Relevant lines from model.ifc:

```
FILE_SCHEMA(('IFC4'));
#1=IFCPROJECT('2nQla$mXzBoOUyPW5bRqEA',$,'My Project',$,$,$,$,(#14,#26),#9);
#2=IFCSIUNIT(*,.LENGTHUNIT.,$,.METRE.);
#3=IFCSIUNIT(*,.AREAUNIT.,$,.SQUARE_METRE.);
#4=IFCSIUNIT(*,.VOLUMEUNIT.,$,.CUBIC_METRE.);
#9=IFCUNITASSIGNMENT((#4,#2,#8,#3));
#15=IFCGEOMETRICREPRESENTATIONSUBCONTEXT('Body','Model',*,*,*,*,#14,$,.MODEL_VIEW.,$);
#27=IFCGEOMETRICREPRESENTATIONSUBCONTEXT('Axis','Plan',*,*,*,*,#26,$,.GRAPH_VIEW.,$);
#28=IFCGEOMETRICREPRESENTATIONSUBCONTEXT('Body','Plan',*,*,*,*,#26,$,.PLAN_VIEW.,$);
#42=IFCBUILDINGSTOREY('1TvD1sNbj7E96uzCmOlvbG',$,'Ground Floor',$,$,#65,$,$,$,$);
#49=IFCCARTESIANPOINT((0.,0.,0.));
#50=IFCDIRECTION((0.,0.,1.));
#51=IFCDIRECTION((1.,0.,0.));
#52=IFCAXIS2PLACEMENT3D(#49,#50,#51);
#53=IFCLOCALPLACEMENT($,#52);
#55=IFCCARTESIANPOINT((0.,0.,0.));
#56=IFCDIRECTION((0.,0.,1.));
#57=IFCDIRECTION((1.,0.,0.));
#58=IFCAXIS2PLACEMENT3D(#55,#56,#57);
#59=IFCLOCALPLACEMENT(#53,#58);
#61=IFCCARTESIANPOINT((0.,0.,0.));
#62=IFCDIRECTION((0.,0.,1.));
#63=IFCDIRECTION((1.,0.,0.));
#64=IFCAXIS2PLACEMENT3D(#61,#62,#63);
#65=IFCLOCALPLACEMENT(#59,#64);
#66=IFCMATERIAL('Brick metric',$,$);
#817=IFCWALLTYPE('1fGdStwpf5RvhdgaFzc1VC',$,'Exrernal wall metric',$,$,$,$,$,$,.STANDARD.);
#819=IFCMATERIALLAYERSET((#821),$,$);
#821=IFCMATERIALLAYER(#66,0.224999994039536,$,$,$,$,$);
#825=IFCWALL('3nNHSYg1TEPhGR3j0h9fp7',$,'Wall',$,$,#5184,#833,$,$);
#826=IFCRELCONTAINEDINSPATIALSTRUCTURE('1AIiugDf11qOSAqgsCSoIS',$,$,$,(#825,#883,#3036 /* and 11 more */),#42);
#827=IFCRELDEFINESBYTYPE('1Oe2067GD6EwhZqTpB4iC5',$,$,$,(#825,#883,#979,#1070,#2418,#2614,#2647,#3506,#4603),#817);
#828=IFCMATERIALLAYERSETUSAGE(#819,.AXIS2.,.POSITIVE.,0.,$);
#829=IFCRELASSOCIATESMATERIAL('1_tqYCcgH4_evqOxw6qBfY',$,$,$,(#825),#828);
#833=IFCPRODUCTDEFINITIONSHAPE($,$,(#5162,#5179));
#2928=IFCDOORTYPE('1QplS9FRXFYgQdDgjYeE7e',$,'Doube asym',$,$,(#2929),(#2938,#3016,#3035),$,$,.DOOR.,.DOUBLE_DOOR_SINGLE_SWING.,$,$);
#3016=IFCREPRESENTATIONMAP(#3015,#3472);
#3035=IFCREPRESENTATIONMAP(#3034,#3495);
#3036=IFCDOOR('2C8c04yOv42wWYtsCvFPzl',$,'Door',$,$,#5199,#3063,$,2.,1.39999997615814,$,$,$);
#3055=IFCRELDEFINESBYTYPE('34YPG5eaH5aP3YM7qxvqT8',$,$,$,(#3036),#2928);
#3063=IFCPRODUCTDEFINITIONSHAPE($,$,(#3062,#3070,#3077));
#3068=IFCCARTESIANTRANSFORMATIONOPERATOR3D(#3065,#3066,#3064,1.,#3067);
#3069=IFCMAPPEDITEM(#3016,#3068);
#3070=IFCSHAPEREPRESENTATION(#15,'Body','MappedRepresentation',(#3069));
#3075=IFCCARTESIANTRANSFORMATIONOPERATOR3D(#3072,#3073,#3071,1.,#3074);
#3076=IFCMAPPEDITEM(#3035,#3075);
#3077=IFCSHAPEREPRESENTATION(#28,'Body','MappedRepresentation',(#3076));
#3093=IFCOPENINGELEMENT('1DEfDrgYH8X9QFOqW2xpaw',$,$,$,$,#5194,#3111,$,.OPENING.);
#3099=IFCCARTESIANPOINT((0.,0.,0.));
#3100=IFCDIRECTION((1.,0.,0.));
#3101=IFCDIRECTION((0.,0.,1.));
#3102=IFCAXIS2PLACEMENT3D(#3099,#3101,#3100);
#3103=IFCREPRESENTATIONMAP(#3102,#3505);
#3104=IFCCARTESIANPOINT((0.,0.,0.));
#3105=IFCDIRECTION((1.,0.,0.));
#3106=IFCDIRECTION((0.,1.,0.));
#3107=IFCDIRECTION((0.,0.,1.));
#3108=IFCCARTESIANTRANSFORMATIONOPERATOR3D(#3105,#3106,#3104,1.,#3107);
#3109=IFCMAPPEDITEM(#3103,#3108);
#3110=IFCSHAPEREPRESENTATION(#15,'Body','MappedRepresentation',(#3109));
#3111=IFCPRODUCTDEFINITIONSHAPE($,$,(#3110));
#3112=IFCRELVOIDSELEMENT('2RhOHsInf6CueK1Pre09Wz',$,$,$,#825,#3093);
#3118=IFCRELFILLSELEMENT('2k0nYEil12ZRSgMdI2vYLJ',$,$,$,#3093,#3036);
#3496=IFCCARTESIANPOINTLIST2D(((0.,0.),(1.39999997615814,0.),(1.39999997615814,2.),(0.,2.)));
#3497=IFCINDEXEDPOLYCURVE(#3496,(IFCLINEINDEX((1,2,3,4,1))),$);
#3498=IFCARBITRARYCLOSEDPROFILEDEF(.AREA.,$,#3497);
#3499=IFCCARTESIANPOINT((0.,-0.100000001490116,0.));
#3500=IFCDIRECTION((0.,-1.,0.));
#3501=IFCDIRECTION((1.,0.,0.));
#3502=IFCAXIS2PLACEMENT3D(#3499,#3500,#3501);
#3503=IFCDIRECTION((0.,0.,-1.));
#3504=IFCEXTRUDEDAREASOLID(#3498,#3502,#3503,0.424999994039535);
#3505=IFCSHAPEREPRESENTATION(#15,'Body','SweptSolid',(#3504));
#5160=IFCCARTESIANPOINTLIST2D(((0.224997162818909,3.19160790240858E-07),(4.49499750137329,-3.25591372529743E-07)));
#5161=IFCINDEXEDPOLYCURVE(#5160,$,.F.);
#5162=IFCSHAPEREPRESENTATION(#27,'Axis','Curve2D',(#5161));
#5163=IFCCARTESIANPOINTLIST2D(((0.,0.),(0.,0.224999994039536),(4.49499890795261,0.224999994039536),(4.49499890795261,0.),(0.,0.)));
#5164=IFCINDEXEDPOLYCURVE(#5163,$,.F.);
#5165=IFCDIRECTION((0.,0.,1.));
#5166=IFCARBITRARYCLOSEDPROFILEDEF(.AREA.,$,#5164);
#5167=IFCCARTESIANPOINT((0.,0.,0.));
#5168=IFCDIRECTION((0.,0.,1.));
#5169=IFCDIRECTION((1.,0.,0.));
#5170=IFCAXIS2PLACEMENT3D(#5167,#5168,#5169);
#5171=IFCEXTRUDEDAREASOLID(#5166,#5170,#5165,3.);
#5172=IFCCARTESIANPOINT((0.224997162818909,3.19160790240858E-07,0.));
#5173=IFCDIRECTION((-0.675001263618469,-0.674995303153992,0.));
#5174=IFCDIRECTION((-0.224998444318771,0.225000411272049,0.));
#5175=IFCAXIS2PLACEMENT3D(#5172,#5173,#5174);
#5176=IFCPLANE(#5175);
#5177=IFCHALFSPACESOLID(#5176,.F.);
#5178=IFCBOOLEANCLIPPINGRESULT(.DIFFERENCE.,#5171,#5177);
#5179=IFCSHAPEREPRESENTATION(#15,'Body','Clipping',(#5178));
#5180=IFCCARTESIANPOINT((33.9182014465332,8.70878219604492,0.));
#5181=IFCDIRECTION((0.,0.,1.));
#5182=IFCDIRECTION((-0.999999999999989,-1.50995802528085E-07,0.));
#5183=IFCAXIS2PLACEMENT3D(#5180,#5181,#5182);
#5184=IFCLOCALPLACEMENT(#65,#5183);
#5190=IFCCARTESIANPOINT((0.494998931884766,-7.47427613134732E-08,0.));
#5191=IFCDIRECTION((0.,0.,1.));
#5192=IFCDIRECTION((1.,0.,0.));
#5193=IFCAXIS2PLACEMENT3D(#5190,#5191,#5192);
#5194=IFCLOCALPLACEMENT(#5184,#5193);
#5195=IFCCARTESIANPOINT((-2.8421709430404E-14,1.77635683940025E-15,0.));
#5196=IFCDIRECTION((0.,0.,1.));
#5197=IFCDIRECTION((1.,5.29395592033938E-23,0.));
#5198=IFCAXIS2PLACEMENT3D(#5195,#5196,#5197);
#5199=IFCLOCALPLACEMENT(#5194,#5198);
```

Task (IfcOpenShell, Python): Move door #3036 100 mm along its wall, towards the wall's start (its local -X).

```python
import ifcopenshell
import ifcopenshell.api.geometry
import ifcopenshell.util.placement

model = ifcopenshell.open("model.ifc")

door = model.by_guid("2C8c04yOv42wWYtsCvFPzl")
opening = door.FillsVoids[0].RelatingOpeningElement
wall = opening.VoidsElements[0].RelatingBuildingElement

wall_matrix = ifcopenshell.util.placement.get_local_placement(wall.ObjectPlacement)
shift = wall_matrix[:3, 0] * -0.1
before = ifcopenshell.util.placement.get_local_placement(door.ObjectPlacement)[:3, 3].copy()

# The door is placed relative to its opening, so it follows when the opening moves.
matrix = ifcopenshell.util.placement.get_local_placement(opening.ObjectPlacement)
matrix[:3, 3] += shift
ifcopenshell.api.geometry.edit_object_placement(
    model, product=opening, matrix=matrix, is_si=False, should_transform_children=True
)

after = ifcopenshell.util.placement.get_local_placement(door.ObjectPlacement)[:3, 3]
print("door moved by", (after - before).round(3) + 0.0)

model.write("model_v2.ifc")
```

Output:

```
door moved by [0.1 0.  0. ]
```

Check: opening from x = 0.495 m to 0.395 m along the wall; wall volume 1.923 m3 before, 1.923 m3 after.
